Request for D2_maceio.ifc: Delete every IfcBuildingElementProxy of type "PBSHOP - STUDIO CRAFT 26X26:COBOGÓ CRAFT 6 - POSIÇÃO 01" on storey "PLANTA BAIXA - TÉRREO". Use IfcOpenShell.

First a look at what the model holds.

```python
import ifcopenshell
import ifcopenshell.util.element

model = ifcopenshell.open("D2_maceio.ifc")
print(model.schema)
storey = next(s for s in model.by_type("IfcBuildingStorey") if s.Name == "PLANTA BAIXA - TÉRREO")
proxies = [e for e in ifcopenshell.util.element.get_decomposition(storey) if e.is_a("IfcBuildingElementProxy")]
seen = {}
for e in proxies:
    element_type = ifcopenshell.util.element.get_type(e)
    name = element_type.Name if element_type not in (None, e) else None
    seen[name] = seen.get(name, 0) + 1
for name, count in sorted(seen.items(), key=str):
    print(count, "x", name)
```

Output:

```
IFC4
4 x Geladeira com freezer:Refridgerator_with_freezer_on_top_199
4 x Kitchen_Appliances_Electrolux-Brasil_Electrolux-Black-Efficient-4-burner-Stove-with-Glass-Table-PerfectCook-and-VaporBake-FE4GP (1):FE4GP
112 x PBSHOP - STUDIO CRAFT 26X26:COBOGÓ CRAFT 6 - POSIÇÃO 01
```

```python
import ifcopenshell
import ifcopenshell.api.root
import ifcopenshell.util.element

model = ifcopenshell.open("D2_maceio.ifc")

storey = next(s for s in model.by_type("IfcBuildingStorey") if s.Name == "PLANTA BAIXA - TÉRREO")
proxies = [e for e in ifcopenshell.util.element.get_decomposition(storey) if e.is_a("IfcBuildingElementProxy")]
targets = [e for e in proxies if (t := ifcopenshell.util.element.get_type(e)) not in (None, e) and t.Name == "PBSHOP - STUDIO CRAFT 26X26:COBOGÓ CRAFT 6 - POSIÇÃO 01"]

for e in targets:
    ifcopenshell.api.root.remove_product(model, product=e)
print(len(targets), "removed")

model.write("D2_maceio-out.ifc")
```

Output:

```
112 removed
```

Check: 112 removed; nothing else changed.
